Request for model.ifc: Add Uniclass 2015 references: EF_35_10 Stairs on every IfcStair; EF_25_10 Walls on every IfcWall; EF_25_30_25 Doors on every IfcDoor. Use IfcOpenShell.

First a look at what the model holds.

```python
import ifcopenshell

model = ifcopenshell.open("model.ifc")
print(model.schema)
print("classifications:", [c.Name for c in model.by_type("IfcClassification")])
for ifc_class in ("IfcDoor", "IfcRoof", "IfcStair", "IfcWall", "IfcWindow"):
    print(ifc_class, len(model.by_type(ifc_class)))
```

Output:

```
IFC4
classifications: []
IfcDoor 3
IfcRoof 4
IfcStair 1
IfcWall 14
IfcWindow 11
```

```python
import ifcopenshell
import ifcopenshell.api.classification

model = ifcopenshell.open("model.ifc")

system = ifcopenshell.api.classification.add_classification(model, classification="Uniclass 2015")

codes = {
    "IfcStair": ("EF_35_10", "Stairs"),
    "IfcWall": ("EF_25_10", "Walls"),
    "IfcDoor": ("EF_25_30_25", "Doors"),
}
for ifc_class, (code, name) in codes.items():
    products = model.by_type(ifc_class)
    ifcopenshell.api.classification.add_reference(
        model, products=products, classification=system, identification=code, name=name
    )
    print(code, len(products))

model.write("model_updated.ifc")
```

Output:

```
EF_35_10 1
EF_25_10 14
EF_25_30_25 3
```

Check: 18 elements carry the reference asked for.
